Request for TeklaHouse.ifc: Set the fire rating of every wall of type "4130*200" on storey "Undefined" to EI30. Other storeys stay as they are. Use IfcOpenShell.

First a look at what the model holds.

```python
import ifcopenshell
import ifcopenshell.util.element

model = ifcopenshell.open("TeklaHouse.ifc")
print(model.schema)
storey = next(s for s in model.by_type("IfcBuildingStorey") if s.Name == "Undefined")
walls = [e for e in ifcopenshell.util.element.get_decomposition(storey) if e.is_a("IfcWall")]
seen = {}
for e in walls:
    element_type = ifcopenshell.util.element.get_type(e)
    key = (element_type.Name if element_type != e and element_type else None, ifcopenshell.util.element.get_pset(e, "Pset_WallCommon", "FireRating"))
    seen[key] = seen.get(key, 0) + 1
for (name, value), count in sorted(seen.items(), key=str):
    print(count, "x", name, "|", value)
```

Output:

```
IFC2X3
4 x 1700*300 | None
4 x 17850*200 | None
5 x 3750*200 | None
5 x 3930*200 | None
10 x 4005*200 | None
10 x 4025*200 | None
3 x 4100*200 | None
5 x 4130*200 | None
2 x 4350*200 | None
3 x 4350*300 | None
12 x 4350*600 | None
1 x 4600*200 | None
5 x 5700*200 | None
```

```python
import ifcopenshell
import ifcopenshell.api.pset
import ifcopenshell.util.element

model = ifcopenshell.open("TeklaHouse.ifc")

storey = next(s for s in model.by_type("IfcBuildingStorey") if s.Name == "Undefined")
walls = [e for e in ifcopenshell.util.element.get_decomposition(storey) if e.is_a("IfcWall")]

count = 0
for e in walls:
    element_type = ifcopenshell.util.element.get_type(e)
    if element_type in (None, e) or element_type.Name != "4130*200":
        continue
    # add_pset returns the element's existing set when there is one.
    pset = ifcopenshell.api.pset.add_pset(model, product=e, name="Pset_WallCommon")
    ifcopenshell.api.pset.edit_pset(model, pset=pset, properties={"FireRating": "EI30"})
    count += 1

print(count, "walls updated")

model.write("TeklaHouse_updated.ifc")
```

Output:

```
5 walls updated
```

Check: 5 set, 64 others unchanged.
